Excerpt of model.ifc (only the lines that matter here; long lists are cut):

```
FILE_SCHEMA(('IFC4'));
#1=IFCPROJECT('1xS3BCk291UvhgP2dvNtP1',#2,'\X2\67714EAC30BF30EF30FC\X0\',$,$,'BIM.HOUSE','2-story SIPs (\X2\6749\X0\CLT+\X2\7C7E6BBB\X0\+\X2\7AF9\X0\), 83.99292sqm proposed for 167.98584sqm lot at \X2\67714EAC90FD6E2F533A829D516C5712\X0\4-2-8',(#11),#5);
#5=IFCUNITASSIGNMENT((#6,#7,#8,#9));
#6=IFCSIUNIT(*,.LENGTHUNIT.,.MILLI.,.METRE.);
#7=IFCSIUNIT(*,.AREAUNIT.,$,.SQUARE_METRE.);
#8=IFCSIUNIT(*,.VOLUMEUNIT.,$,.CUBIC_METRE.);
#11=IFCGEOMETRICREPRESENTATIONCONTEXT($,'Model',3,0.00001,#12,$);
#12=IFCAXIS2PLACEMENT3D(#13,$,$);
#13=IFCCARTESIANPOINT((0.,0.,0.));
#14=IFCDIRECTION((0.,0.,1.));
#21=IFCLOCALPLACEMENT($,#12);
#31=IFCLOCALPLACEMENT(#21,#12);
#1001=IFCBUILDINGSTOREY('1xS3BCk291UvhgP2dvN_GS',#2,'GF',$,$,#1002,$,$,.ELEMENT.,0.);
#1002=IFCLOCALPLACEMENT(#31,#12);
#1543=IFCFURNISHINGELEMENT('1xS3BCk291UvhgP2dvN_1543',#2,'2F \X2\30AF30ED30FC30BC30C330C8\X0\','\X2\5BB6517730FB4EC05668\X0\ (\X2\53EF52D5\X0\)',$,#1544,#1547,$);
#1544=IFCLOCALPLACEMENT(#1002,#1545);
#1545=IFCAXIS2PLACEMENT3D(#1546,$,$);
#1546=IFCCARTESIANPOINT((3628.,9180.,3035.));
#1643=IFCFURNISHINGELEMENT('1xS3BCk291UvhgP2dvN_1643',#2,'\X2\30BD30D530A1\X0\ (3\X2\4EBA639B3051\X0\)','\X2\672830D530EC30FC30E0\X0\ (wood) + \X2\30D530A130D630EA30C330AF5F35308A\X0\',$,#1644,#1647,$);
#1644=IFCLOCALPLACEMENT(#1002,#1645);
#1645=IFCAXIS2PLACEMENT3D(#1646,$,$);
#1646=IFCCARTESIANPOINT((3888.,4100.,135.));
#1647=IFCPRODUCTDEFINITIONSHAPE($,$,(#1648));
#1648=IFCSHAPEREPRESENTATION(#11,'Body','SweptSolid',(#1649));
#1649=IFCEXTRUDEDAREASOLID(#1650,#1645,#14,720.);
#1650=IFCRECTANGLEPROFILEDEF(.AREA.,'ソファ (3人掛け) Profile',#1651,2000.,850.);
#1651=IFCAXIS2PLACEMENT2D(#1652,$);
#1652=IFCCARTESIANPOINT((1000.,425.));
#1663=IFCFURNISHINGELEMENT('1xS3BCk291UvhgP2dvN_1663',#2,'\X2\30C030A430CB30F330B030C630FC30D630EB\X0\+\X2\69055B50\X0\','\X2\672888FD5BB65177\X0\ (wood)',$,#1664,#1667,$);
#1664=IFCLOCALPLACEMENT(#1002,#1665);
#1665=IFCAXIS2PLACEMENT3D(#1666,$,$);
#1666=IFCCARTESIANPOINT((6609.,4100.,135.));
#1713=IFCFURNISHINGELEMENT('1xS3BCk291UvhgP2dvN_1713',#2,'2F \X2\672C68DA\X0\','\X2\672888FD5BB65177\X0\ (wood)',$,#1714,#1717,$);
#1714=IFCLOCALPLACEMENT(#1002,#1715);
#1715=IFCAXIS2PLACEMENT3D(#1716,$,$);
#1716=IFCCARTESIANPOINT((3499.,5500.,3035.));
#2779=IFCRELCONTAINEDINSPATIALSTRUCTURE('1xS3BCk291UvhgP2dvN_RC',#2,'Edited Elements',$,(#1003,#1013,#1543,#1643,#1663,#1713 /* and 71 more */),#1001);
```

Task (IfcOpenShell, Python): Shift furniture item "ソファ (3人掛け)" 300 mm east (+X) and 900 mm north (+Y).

```python
import ifcopenshell
import ifcopenshell.api.geometry
import ifcopenshell.util.placement

model = ifcopenshell.open("model.ifc")

item = model.by_guid("1xS3BCk291UvhgP2dvN_1643")
matrix = ifcopenshell.util.placement.get_local_placement(item.ObjectPlacement)
matrix[0, 3] += 300.0
matrix[1, 3] += 900.0
ifcopenshell.api.geometry.edit_object_placement(model, product=item, matrix=matrix, is_si=False)

print(ifcopenshell.util.placement.get_local_placement(item.ObjectPlacement).round(3) + 0.0)

model.write("model_rev.ifc")
```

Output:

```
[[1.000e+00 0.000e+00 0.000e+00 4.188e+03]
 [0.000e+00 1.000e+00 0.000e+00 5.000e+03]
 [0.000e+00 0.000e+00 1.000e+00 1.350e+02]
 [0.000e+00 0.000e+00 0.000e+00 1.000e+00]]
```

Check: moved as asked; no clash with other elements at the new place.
